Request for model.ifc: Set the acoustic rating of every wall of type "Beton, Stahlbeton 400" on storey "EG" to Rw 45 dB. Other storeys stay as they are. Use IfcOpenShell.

First a look at what the model holds.

```python
import ifcopenshell
import ifcopenshell.util.element

model = ifcopenshell.open("model.ifc")
print(model.schema)
storey = next(s for s in model.by_type("IfcBuildingStorey") if s.Name == "EG")
walls = [e for e in ifcopenshell.util.element.get_decomposition(storey) if e.is_a("IfcWall")]
seen = {}
for e in walls:
    element_type = ifcopenshell.util.element.get_type(e)
    key = (element_type.Name if element_type != e and element_type else None, ifcopenshell.util.element.get_pset(e, "Pset_WallCommon", "AcousticRating"))
    seen[key] = seen.get(key, 0) + 1
for (name, value), count in sorted(seen.items(), key=str):
    print(count, "x", name, "|", value)
```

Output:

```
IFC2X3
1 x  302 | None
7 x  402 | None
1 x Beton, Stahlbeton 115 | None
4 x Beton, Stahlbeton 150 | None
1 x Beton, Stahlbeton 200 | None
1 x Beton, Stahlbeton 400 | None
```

```python
import ifcopenshell
import ifcopenshell.api.pset
import ifcopenshell.util.element

model = ifcopenshell.open("model.ifc")

storey = next(s for s in model.by_type("IfcBuildingStorey") if s.Name == "EG")
walls = [e for e in ifcopenshell.util.element.get_decomposition(storey) if e.is_a("IfcWall")]

count = 0
for e in walls:
    element_type = ifcopenshell.util.element.get_type(e)
    if element_type in (None, e) or element_type.Name != "Beton, Stahlbeton 400":
        continue
    # add_pset returns the element's existing set when there is one.
    pset = ifcopenshell.api.pset.add_pset(model, product=e, name="Pset_WallCommon")
    ifcopenshell.api.pset.edit_pset(model, pset=pset, properties={"AcousticRating": "Rw 45 dB"})
    count += 1

print(count, "walls updated")

model.write("model_v2.ifc")
```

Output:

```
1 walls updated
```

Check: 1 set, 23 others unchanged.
